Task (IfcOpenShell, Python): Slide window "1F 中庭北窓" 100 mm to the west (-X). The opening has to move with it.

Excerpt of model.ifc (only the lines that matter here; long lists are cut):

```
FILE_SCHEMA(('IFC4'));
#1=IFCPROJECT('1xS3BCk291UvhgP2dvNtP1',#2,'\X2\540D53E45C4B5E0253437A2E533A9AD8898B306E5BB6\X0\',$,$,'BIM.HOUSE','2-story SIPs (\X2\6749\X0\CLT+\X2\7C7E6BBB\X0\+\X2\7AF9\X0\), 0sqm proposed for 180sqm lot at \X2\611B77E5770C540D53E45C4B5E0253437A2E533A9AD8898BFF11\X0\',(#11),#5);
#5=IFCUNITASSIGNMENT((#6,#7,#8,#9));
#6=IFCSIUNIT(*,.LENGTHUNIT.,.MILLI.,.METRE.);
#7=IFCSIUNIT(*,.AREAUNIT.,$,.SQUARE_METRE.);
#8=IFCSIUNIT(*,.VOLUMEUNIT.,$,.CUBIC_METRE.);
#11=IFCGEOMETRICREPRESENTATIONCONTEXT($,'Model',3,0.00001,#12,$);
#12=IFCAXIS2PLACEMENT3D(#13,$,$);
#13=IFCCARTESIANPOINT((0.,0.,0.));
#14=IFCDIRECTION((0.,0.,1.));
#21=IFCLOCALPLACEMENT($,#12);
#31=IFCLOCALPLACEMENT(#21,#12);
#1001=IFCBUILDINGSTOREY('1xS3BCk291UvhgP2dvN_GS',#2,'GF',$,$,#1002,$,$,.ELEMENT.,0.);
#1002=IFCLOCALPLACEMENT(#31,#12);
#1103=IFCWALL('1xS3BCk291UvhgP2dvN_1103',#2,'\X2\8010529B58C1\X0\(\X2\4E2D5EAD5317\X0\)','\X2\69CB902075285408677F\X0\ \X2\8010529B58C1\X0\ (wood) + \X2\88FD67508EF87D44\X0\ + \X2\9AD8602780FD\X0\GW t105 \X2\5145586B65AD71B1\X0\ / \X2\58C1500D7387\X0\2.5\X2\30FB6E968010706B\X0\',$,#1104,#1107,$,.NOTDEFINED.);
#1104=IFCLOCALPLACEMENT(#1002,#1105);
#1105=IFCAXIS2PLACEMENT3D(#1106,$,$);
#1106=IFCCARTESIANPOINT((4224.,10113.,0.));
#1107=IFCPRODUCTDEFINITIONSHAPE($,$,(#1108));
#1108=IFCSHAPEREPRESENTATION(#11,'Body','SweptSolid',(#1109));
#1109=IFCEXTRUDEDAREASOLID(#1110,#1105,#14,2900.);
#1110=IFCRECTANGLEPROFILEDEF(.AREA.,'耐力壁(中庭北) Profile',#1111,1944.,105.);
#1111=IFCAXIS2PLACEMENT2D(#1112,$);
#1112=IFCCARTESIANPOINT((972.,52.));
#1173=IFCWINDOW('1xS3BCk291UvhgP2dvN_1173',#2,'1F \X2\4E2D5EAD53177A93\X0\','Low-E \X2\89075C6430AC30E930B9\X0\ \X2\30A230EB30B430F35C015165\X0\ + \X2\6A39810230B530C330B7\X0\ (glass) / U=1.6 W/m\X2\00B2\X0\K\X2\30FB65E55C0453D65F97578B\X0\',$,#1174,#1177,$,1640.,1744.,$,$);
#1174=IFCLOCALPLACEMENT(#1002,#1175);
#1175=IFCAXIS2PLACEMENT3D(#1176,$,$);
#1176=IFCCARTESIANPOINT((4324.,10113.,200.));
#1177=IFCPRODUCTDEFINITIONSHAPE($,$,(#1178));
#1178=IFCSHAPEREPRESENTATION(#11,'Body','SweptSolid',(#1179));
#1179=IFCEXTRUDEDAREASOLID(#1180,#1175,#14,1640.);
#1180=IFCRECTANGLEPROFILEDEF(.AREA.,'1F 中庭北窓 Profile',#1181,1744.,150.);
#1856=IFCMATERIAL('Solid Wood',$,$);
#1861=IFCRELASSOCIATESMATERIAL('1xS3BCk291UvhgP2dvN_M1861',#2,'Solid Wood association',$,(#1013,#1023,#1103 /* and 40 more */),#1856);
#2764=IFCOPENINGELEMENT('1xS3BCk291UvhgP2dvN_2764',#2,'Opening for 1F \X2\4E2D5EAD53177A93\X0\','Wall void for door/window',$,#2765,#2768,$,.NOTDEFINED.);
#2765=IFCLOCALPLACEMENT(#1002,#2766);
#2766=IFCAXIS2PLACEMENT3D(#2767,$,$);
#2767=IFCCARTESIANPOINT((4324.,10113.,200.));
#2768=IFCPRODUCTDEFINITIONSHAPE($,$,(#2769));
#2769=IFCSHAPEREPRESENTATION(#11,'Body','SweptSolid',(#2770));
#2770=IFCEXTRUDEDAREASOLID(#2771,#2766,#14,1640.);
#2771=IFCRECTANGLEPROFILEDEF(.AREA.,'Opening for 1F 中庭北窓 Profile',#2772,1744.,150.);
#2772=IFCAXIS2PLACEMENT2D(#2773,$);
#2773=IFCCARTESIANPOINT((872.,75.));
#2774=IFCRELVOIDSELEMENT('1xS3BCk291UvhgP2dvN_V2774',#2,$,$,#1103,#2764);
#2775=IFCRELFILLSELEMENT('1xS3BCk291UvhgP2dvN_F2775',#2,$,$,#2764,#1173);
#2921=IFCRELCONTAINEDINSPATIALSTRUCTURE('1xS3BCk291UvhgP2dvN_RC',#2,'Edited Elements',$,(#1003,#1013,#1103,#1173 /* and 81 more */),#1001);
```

```python
import ifcopenshell
import ifcopenshell.api.geometry
import ifcopenshell.util.placement
import ifcopenshell.util.unit

model = ifcopenshell.open("model.ifc")
unit_scale = ifcopenshell.util.unit.calculate_unit_scale(model)

window = model.by_guid("1xS3BCk291UvhgP2dvN_1173")
opening = window.FillsVoids[0].RelatingOpeningElement
wall = opening.VoidsElements[0].RelatingBuildingElement

wall_matrix = ifcopenshell.util.placement.get_local_placement(wall.ObjectPlacement)
shift = wall_matrix[:3, 0] * -0.1 / unit_scale
before = ifcopenshell.util.placement.get_local_placement(window.ObjectPlacement)[:3, 3].copy()

# The window is not placed relative to its opening, so move both.
for product in (opening, window):
    matrix = ifcopenshell.util.placement.get_local_placement(product.ObjectPlacement)
    matrix[:3, 3] += shift
    ifcopenshell.api.geometry.edit_object_placement(model, product=product, matrix=matrix, is_si=False)

after = ifcopenshell.util.placement.get_local_placement(window.ObjectPlacement)[:3, 3]
print("window moved by", (after - before).round(3) + 0.0)

model.write("model_edited.ifc")
```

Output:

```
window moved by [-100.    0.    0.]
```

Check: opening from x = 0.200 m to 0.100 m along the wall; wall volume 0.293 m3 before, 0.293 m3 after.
